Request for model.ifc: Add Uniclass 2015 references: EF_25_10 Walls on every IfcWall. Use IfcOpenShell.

First a look at what the model holds.

```python
import ifcopenshell

model = ifcopenshell.open("model.ifc")
print(model.schema)
print("classifications:", [c.Name for c in model.by_type("IfcClassification")])
for ifc_class in ("IfcDoor", "IfcRoof", "IfcStair", "IfcWall", "IfcWindow"):
    print(ifc_class, len(model.by_type(ifc_class)))
```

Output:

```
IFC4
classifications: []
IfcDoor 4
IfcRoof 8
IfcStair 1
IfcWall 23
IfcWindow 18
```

```python
import ifcopenshell
import ifcopenshell.api.classification

model = ifcopenshell.open("model.ifc")

system = ifcopenshell.api.classification.add_classification(model, classification="Uniclass 2015")

codes = {
    "IfcWall": ("EF_25_10", "Walls"),
}
for ifc_class, (code, name) in codes.items():
    products = model.by_type(ifc_class)
    ifcopenshell.api.classification.add_reference(
        model, products=products, classification=system, identification=code, name=name
    )
    print(code, len(products))

model.write("model-out.ifc")
```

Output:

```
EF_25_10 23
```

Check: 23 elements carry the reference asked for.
